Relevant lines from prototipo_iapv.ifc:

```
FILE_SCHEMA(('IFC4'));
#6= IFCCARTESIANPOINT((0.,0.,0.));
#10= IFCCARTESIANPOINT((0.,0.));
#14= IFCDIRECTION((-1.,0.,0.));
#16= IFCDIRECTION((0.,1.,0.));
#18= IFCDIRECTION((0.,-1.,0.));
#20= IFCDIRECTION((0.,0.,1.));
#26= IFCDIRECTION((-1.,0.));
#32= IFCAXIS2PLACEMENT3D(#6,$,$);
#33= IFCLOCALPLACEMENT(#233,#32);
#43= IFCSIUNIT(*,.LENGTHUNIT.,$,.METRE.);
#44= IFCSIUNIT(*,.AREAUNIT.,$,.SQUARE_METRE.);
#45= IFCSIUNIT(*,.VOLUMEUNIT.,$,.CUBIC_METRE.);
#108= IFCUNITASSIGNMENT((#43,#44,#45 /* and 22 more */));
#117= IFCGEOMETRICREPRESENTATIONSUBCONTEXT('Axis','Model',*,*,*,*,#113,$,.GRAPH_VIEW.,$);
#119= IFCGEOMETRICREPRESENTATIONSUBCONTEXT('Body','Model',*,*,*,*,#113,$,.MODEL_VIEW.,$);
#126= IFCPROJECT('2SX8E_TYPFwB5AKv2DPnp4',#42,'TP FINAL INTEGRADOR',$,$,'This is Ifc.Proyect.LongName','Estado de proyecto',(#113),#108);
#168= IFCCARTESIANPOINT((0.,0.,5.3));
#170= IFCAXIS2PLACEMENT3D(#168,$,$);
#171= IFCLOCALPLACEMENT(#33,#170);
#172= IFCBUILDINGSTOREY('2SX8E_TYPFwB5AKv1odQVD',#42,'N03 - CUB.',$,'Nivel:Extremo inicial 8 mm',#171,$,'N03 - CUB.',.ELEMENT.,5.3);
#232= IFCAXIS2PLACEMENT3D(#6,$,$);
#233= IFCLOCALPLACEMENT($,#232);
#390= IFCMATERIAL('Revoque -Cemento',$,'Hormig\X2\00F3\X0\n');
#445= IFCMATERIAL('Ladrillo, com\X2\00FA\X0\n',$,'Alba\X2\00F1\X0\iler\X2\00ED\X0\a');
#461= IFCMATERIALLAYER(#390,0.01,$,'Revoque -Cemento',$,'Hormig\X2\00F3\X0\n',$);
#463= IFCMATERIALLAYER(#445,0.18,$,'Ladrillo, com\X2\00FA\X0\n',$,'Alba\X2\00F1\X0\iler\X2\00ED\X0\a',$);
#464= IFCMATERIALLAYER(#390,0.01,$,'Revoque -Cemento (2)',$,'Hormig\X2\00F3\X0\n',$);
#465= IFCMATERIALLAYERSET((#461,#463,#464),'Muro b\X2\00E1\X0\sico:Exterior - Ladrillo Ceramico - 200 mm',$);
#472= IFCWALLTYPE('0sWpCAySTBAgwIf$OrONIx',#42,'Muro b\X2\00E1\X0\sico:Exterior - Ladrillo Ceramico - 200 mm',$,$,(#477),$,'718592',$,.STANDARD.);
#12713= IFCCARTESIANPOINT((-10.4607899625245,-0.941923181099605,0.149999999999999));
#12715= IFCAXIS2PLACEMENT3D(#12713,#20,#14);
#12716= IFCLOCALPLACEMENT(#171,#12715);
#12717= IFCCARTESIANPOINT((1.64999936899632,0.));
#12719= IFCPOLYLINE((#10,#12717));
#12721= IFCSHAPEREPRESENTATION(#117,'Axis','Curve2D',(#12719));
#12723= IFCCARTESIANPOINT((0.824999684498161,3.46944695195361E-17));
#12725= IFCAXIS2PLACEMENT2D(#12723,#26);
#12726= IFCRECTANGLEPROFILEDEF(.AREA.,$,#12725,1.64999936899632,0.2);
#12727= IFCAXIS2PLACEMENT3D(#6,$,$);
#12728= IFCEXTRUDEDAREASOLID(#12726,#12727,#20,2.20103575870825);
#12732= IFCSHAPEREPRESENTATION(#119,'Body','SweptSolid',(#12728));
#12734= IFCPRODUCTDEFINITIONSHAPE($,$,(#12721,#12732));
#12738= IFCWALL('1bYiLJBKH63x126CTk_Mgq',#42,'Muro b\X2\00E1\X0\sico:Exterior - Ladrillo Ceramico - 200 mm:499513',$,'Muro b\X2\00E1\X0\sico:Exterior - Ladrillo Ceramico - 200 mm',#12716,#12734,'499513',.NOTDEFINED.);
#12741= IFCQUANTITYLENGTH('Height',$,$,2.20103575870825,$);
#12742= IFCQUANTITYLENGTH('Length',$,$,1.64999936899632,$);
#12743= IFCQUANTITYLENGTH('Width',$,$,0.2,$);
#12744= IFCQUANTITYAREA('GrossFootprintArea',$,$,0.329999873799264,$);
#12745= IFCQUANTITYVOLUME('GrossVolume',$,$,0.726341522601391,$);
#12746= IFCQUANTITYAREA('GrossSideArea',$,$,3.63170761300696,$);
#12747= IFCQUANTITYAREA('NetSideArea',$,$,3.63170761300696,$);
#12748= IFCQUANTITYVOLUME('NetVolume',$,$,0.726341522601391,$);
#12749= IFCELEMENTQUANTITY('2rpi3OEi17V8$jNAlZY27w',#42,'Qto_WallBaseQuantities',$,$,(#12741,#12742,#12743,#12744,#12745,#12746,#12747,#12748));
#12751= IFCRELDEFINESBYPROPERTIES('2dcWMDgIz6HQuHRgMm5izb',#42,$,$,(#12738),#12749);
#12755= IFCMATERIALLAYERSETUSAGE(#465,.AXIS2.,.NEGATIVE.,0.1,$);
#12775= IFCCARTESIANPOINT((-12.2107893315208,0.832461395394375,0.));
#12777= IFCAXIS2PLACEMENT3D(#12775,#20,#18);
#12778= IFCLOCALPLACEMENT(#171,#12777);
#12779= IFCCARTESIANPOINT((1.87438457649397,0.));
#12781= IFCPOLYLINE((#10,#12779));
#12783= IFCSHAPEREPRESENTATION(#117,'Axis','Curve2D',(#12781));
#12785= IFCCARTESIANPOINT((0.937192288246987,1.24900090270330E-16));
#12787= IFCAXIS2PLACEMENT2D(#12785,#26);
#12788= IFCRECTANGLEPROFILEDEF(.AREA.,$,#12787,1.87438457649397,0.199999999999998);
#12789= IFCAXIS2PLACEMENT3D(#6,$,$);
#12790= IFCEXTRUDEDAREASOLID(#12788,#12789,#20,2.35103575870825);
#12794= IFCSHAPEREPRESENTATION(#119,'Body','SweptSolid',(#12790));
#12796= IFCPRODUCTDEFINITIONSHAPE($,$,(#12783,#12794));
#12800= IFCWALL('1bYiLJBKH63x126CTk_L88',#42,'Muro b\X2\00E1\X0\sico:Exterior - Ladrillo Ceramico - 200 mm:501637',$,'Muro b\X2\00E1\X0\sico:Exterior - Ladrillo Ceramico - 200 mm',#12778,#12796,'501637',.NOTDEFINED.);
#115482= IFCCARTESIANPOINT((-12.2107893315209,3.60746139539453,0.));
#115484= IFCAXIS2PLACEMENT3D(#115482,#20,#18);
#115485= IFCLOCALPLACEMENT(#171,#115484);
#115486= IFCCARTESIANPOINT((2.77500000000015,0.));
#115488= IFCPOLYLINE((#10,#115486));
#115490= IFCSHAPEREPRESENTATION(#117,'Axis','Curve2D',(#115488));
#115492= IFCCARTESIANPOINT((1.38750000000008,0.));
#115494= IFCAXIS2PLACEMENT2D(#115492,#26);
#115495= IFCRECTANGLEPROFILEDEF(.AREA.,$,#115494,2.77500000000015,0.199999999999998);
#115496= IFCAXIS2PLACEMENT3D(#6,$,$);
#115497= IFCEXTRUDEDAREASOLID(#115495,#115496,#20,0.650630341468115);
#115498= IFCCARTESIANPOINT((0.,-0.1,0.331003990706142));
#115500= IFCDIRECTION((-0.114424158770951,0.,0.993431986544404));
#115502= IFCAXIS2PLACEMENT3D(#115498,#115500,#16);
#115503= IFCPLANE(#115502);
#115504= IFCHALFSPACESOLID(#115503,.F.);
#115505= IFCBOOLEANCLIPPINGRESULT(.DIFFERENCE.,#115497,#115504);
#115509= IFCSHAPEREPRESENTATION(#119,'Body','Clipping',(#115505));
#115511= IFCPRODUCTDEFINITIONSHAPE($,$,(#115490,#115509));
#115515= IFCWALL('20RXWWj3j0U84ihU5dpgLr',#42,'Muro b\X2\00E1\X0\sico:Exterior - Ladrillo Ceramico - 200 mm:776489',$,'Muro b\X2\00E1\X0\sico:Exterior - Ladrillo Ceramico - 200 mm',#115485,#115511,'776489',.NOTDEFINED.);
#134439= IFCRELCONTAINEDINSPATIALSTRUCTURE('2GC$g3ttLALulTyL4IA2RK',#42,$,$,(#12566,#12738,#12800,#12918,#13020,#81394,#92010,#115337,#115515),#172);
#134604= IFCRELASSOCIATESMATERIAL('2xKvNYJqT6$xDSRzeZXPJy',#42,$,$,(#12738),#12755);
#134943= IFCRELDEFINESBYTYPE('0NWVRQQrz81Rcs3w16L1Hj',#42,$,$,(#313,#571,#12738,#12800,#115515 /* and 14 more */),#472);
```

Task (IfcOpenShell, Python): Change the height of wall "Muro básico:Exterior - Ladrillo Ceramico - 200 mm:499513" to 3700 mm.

```python
import ifcopenshell
import ifcopenshell.api.pset
import ifcopenshell.geom
import ifcopenshell.util.element
import ifcopenshell.util.representation
import ifcopenshell.util.shape
import ifcopenshell.util.unit

model = ifcopenshell.open("prototipo_iapv.ifc")
unit_scale = ifcopenshell.util.unit.calculate_unit_scale(model)
area_scale = ifcopenshell.util.unit.calculate_unit_scale(model, "AREAUNIT")
volume_scale = ifcopenshell.util.unit.calculate_unit_scale(model, "VOLUMEUNIT")
settings = ifcopenshell.geom.settings()


def volume(element):
    """Net volume in cubic metres, openings subtracted."""
    shape = ifcopenshell.geom.create_shape(settings, element)
    return ifcopenshell.util.shape.get_volume(shape.geometry)


wall = model.by_id(12738)
before = volume(wall)

body = ifcopenshell.util.representation.get_representation(wall, "Model", "Body")
solid = body.Items[0]
old_height = solid.Depth
solid.Depth = 3.7 / unit_scale
after = volume(wall)
thickness = 0.2  # wall thickness in metres

# Update the stored height, areas and volumes.
qto = model.by_id(ifcopenshell.util.element.get_pset(wall, "Qto_WallBaseQuantities", should_inherit=False)["id"])
ifcopenshell.api.pset.edit_qto(model, qto=qto, properties={
    "Height": solid.Depth,
    "GrossVolume": ifcopenshell.util.element.get_pset(wall, "Qto_WallBaseQuantities", "GrossVolume") * solid.Depth / old_height,
    "GrossSideArea": ifcopenshell.util.element.get_pset(wall, "Qto_WallBaseQuantities", "GrossSideArea") * solid.Depth / old_height,
    "NetSideArea": after / thickness / area_scale,
    "NetVolume": after / volume_scale,
})

print(f"height {old_height:g} -> {solid.Depth:g}, volume {before:.3f} -> {after:.3f} m3")

model.write("prototipo_iapv_v2.ifc")
```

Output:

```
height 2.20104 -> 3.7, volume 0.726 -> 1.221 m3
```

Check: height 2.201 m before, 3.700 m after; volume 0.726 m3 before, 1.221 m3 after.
